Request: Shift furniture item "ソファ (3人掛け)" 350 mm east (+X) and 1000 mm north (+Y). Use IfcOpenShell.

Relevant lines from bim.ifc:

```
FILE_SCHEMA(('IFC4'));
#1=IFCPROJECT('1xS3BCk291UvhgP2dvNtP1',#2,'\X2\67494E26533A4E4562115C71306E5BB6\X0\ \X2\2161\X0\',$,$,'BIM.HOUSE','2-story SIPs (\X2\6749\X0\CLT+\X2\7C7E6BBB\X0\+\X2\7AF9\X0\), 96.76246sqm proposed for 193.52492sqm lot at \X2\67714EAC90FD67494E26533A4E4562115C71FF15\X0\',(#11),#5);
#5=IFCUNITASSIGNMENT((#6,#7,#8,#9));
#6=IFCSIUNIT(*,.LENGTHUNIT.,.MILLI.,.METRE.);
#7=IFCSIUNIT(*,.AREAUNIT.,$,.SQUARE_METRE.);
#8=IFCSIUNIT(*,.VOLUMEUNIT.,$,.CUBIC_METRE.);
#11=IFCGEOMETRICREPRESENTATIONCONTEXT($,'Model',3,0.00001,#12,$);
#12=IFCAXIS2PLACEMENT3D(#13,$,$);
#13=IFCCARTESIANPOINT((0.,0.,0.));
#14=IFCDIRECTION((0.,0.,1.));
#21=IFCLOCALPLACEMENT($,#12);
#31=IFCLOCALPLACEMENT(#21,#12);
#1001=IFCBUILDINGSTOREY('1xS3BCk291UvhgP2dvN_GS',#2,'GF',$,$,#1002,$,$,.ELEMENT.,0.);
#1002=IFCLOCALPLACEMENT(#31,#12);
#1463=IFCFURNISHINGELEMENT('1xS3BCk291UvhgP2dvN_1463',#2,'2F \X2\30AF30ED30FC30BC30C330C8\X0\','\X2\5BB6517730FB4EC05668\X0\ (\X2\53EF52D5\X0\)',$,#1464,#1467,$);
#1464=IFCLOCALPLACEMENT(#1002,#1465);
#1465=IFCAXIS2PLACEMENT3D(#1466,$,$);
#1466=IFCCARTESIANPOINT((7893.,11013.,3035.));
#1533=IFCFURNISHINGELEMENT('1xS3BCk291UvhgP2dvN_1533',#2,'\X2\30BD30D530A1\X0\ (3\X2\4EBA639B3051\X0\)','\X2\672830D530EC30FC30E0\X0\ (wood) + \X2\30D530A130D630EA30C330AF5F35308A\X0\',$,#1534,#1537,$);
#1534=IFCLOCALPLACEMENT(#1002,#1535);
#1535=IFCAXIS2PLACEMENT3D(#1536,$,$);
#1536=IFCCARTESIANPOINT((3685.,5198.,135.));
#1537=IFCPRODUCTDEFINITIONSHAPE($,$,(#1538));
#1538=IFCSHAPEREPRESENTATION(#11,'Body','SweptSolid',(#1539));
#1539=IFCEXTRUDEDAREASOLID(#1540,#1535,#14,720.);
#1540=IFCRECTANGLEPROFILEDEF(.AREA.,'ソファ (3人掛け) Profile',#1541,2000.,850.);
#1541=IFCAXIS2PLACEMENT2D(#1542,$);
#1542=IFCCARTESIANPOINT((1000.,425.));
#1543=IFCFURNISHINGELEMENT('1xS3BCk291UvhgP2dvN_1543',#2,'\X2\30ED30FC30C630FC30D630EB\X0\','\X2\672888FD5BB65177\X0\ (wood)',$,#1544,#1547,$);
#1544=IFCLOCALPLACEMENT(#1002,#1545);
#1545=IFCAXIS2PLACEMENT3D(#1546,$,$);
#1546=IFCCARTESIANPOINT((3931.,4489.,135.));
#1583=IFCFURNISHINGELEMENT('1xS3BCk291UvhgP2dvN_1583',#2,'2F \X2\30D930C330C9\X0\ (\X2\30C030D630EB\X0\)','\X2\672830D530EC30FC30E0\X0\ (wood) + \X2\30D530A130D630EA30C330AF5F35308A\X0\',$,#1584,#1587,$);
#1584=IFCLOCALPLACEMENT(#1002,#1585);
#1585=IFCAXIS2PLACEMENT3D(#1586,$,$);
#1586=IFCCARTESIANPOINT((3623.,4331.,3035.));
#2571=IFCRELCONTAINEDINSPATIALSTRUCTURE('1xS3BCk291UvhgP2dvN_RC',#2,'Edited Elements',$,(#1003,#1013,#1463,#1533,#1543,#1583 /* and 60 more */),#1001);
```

```python
import ifcopenshell
import ifcopenshell.api.geometry
import ifcopenshell.util.placement

model = ifcopenshell.open("bim.ifc")

item = model.by_guid("1xS3BCk291UvhgP2dvN_1533")
matrix = ifcopenshell.util.placement.get_local_placement(item.ObjectPlacement)
matrix[0, 3] += 350.0
matrix[1, 3] += 1000.0
ifcopenshell.api.geometry.edit_object_placement(model, product=item, matrix=matrix, is_si=False)

print(ifcopenshell.util.placement.get_local_placement(item.ObjectPlacement).round(3) + 0.0)

model.write("bim_rev.ifc")
```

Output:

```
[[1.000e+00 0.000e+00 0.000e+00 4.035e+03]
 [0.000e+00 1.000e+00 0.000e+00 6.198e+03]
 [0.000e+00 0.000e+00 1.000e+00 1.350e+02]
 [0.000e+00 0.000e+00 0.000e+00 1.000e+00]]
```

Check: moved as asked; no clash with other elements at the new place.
